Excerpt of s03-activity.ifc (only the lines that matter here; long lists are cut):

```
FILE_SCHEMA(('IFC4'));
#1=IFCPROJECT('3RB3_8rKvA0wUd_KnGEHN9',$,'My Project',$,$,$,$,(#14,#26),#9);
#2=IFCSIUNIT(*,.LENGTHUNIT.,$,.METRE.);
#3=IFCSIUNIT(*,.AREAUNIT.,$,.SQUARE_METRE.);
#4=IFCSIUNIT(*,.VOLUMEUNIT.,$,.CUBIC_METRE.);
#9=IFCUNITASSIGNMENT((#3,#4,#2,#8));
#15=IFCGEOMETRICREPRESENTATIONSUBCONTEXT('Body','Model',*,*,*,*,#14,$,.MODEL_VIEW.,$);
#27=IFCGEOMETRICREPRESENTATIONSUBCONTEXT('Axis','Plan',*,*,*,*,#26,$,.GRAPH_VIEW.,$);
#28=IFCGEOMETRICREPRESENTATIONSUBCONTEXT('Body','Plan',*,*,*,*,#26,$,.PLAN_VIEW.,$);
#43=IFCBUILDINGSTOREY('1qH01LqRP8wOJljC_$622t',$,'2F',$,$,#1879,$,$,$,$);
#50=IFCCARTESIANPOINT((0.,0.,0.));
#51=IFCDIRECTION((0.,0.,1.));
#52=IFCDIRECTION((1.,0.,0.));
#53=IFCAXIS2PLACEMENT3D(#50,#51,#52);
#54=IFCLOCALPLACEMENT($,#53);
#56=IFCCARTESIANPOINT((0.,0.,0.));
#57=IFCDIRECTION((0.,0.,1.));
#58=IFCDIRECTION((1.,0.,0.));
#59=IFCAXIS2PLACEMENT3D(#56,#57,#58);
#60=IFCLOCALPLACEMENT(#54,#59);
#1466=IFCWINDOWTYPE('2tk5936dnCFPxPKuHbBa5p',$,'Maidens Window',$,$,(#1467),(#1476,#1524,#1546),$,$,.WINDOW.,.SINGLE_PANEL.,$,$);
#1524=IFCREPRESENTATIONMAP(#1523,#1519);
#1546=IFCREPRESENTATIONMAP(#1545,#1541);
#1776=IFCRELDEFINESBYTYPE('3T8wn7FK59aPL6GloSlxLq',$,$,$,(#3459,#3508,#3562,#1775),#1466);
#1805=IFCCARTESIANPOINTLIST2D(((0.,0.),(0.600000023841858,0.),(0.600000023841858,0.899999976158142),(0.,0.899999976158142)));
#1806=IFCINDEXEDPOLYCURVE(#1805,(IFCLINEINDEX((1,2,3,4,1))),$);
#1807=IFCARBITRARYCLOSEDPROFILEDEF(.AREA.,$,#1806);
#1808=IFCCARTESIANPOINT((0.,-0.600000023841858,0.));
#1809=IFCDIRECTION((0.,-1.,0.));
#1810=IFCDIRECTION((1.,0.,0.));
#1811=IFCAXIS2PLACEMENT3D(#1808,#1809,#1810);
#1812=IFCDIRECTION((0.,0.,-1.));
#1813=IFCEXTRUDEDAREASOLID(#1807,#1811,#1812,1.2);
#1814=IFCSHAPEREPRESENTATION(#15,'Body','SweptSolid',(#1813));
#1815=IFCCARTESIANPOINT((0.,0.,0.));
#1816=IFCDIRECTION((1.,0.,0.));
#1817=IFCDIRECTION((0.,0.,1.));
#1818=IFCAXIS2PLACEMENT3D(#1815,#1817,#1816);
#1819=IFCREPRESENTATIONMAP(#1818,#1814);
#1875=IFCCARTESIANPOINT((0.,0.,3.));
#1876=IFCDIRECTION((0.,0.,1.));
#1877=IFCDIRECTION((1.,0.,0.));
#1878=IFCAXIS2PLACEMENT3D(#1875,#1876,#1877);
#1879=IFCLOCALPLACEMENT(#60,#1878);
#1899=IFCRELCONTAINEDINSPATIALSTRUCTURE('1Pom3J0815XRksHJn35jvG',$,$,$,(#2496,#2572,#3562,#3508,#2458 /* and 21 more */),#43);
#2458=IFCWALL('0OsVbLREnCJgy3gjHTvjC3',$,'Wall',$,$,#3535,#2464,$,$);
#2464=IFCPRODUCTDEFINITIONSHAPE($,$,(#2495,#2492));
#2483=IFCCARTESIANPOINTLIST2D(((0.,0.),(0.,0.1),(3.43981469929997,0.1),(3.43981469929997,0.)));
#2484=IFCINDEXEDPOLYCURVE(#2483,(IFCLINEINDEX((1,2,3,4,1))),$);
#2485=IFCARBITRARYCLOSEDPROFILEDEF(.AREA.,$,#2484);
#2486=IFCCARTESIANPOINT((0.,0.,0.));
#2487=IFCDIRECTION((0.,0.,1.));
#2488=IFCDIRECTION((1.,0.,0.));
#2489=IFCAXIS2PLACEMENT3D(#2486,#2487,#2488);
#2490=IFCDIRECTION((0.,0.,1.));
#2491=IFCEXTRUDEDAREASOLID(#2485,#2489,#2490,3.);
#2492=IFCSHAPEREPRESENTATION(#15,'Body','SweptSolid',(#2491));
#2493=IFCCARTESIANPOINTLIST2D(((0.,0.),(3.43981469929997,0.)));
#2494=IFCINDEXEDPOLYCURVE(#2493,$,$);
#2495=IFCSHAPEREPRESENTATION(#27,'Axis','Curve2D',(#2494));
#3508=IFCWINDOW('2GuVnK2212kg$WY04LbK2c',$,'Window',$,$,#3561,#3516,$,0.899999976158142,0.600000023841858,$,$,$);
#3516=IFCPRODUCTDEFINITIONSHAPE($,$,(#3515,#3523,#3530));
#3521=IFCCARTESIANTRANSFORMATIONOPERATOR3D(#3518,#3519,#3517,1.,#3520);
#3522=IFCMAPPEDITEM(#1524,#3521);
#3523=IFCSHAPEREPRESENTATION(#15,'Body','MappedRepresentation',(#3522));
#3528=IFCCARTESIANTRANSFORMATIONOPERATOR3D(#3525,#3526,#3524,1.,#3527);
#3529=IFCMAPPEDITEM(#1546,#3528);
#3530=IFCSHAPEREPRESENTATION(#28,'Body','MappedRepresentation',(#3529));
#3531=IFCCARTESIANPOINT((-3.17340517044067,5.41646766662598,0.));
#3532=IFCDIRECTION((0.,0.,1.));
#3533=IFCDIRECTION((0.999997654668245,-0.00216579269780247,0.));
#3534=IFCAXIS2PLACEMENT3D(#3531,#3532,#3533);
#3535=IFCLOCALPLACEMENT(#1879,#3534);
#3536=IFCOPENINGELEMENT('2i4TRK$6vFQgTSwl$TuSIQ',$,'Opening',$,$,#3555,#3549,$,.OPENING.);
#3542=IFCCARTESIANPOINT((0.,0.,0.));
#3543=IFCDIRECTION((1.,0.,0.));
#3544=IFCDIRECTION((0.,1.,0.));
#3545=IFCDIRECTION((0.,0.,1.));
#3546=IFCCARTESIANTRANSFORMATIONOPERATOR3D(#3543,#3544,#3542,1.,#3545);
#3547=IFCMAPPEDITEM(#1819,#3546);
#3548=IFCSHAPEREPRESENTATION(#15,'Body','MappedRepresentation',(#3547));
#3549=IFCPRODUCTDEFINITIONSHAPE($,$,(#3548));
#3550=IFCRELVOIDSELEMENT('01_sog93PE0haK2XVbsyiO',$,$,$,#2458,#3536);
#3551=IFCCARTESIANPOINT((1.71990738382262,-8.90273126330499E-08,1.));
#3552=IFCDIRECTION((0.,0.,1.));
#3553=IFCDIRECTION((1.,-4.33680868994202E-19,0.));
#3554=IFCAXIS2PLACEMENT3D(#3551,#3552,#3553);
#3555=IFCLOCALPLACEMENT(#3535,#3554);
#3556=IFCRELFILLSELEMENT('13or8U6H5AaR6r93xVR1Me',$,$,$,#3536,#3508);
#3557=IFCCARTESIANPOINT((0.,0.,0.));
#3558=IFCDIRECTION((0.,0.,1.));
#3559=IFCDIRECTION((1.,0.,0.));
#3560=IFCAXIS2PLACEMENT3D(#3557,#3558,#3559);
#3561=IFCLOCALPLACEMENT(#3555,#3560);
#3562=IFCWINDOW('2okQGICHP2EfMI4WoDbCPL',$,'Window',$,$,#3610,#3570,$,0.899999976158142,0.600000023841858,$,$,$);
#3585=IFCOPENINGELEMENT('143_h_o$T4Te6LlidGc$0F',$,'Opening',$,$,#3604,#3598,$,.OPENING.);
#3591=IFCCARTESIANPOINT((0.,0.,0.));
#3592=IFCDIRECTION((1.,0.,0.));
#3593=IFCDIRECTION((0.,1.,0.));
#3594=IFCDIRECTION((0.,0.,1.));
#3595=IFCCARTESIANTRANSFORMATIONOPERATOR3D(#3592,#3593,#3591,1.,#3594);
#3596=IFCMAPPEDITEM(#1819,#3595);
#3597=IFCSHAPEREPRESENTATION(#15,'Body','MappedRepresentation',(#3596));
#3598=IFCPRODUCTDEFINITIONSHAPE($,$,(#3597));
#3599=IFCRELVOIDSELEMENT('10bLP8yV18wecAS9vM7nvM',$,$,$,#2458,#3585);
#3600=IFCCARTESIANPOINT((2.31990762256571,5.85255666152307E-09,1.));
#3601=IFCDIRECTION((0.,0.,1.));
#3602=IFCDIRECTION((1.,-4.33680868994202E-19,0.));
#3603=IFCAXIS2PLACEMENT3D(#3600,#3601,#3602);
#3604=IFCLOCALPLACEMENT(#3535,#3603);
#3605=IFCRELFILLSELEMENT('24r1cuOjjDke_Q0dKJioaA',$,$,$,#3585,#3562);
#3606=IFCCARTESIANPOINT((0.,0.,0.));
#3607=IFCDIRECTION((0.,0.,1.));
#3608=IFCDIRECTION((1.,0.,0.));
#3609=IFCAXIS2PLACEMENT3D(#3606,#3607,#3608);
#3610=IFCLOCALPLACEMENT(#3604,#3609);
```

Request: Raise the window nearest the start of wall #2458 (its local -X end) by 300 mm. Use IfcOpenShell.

```python
import numpy as np
import ifcopenshell
import ifcopenshell.api.geometry
import ifcopenshell.util.placement
import ifcopenshell.util.unit

model = ifcopenshell.open("s03-activity.ifc")
unit_scale = ifcopenshell.util.unit.calculate_unit_scale(model)

window = model.by_guid("2GuVnK2212kg$WY04LbK2c")
opening = window.FillsVoids[0].RelatingOpeningElement
dz = 0.3 / unit_scale

shift = np.array([0.0, 0.0, dz])
# The window is placed relative to its opening, so it follows when the opening moves.
matrix = ifcopenshell.util.placement.get_local_placement(opening.ObjectPlacement)
matrix[:3, 3] += shift
ifcopenshell.api.geometry.edit_object_placement(
    model, product=opening, matrix=matrix, is_si=False, should_transform_children=True
)

print(f"moved by {dz * unit_scale:+.3f} m")

model.write("s03-activity_rev.ifc")
```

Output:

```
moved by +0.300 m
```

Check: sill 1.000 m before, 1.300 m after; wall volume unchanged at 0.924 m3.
